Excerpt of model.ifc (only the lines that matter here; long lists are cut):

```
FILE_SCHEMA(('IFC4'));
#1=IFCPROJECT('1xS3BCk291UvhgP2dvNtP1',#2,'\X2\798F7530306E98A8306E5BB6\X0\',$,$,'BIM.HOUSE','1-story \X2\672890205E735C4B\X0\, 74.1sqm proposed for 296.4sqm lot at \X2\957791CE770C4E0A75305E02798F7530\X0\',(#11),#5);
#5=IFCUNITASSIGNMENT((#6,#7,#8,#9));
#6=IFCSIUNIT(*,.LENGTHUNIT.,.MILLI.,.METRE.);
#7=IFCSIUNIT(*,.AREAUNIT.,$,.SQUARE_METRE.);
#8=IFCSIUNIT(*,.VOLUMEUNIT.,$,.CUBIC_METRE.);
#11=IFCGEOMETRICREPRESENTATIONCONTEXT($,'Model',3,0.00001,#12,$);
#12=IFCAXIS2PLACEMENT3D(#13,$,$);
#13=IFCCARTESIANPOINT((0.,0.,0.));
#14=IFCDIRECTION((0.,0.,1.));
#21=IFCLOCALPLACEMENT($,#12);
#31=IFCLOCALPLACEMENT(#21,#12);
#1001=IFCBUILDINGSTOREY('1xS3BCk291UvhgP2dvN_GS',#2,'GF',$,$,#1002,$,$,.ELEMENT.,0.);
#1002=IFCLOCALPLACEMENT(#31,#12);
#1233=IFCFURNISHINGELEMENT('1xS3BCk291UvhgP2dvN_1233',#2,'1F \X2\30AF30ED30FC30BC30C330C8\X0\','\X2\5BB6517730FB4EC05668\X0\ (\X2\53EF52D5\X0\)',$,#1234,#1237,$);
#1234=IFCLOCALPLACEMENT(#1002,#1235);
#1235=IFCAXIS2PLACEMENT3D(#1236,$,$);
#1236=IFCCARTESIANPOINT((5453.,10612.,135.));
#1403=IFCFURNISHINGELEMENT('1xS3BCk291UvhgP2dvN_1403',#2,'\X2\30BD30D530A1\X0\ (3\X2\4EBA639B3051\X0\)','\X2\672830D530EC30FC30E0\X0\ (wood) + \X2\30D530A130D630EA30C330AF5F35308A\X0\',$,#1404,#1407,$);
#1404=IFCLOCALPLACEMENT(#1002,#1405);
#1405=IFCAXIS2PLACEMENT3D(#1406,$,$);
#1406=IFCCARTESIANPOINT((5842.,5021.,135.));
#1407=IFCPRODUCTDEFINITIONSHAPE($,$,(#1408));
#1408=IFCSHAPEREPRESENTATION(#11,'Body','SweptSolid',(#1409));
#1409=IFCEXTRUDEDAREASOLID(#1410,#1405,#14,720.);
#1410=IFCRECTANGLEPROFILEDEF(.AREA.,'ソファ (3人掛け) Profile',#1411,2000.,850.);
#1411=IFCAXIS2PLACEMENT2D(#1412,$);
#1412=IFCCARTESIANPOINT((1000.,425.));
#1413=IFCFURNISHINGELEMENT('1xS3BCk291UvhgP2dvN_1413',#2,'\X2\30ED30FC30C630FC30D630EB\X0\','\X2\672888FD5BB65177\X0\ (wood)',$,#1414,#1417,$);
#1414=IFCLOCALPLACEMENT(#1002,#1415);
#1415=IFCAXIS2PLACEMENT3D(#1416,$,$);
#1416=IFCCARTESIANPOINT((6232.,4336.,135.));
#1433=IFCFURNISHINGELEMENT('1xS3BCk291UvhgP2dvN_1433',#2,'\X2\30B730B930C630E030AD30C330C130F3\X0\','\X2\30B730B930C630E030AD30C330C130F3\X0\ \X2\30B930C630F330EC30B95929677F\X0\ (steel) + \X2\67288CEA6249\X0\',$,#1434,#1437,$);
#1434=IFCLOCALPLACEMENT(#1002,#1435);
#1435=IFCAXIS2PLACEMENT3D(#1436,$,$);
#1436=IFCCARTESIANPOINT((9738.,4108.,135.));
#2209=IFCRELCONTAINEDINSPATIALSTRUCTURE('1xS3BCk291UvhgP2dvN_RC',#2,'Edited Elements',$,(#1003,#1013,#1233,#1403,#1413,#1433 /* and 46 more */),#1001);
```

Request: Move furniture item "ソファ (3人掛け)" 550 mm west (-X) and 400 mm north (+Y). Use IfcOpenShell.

```python
import ifcopenshell
import ifcopenshell.api.geometry
import ifcopenshell.util.placement
import ifcopenshell.util.unit

model = ifcopenshell.open("model.ifc")
unit_scale = ifcopenshell.util.unit.calculate_unit_scale(model)

item = model.by_guid("1xS3BCk291UvhgP2dvN_1403")
matrix = ifcopenshell.util.placement.get_local_placement(item.ObjectPlacement)
matrix[0, 3] -= 0.55 / unit_scale
matrix[1, 3] += 0.4 / unit_scale
ifcopenshell.api.geometry.edit_object_placement(model, product=item, matrix=matrix, is_si=False)

print(ifcopenshell.util.placement.get_local_placement(item.ObjectPlacement).round(3) + 0.0)

model.write("model-out.ifc")
```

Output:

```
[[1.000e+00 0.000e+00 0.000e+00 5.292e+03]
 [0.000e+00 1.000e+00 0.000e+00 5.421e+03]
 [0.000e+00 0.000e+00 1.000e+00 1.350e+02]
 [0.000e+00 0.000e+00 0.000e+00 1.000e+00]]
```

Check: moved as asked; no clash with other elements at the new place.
